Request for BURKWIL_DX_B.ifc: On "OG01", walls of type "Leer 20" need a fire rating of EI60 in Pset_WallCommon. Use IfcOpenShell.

First a look at what the model holds.

```python
import ifcopenshell
import ifcopenshell.util.element

model = ifcopenshell.open("BURKWIL_DX_B.ifc")
print(model.schema)
storey = next(s for s in model.by_type("IfcBuildingStorey") if s.Name == "OG01")
walls = [e for e in ifcopenshell.util.element.get_decomposition(storey) if e.is_a("IfcWall")]
seen = {}
for e in walls:
    element_type = ifcopenshell.util.element.get_type(e)
    key = (element_type.Name if element_type != e and element_type else None, ifcopenshell.util.element.get_pset(e, "Pset_WallCommon", "FireRating"))
    seen[key] = seen.get(key, 0) + 1
for (name, value), count in sorted(seen.items(), key=str):
    print(count, "x", name, "|", value)
```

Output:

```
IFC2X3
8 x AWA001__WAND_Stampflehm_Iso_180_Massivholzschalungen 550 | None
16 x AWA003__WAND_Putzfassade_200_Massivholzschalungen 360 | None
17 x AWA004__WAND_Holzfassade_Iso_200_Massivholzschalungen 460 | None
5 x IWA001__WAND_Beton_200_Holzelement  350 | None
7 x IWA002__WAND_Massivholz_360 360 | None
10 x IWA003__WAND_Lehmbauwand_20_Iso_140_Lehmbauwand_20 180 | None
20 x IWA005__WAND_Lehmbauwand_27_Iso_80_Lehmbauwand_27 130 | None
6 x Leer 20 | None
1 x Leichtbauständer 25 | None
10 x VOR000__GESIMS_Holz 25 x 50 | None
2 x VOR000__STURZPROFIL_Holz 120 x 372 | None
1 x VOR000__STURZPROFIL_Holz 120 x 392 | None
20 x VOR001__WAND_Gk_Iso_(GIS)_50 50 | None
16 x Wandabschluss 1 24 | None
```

```python
import ifcopenshell
import ifcopenshell.api.pset
import ifcopenshell.util.element

model = ifcopenshell.open("BURKWIL_DX_B.ifc")

storey = next(s for s in model.by_type("IfcBuildingStorey") if s.Name == "OG01")
walls = [e for e in ifcopenshell.util.element.get_decomposition(storey) if e.is_a("IfcWall")]

count = 0
for e in walls:
    element_type = ifcopenshell.util.element.get_type(e)
    if element_type in (None, e) or element_type.Name != "Leer 20":
        continue
    # add_pset returns the element's existing set when there is one.
    pset = ifcopenshell.api.pset.add_pset(model, product=e, name="Pset_WallCommon")
    ifcopenshell.api.pset.edit_pset(model, pset=pset, properties={"FireRating": "EI60"})
    count += 1

print(count, "walls updated")

model.write("BURKWIL_DX_B_updated.ifc")
```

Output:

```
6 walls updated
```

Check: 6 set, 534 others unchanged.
